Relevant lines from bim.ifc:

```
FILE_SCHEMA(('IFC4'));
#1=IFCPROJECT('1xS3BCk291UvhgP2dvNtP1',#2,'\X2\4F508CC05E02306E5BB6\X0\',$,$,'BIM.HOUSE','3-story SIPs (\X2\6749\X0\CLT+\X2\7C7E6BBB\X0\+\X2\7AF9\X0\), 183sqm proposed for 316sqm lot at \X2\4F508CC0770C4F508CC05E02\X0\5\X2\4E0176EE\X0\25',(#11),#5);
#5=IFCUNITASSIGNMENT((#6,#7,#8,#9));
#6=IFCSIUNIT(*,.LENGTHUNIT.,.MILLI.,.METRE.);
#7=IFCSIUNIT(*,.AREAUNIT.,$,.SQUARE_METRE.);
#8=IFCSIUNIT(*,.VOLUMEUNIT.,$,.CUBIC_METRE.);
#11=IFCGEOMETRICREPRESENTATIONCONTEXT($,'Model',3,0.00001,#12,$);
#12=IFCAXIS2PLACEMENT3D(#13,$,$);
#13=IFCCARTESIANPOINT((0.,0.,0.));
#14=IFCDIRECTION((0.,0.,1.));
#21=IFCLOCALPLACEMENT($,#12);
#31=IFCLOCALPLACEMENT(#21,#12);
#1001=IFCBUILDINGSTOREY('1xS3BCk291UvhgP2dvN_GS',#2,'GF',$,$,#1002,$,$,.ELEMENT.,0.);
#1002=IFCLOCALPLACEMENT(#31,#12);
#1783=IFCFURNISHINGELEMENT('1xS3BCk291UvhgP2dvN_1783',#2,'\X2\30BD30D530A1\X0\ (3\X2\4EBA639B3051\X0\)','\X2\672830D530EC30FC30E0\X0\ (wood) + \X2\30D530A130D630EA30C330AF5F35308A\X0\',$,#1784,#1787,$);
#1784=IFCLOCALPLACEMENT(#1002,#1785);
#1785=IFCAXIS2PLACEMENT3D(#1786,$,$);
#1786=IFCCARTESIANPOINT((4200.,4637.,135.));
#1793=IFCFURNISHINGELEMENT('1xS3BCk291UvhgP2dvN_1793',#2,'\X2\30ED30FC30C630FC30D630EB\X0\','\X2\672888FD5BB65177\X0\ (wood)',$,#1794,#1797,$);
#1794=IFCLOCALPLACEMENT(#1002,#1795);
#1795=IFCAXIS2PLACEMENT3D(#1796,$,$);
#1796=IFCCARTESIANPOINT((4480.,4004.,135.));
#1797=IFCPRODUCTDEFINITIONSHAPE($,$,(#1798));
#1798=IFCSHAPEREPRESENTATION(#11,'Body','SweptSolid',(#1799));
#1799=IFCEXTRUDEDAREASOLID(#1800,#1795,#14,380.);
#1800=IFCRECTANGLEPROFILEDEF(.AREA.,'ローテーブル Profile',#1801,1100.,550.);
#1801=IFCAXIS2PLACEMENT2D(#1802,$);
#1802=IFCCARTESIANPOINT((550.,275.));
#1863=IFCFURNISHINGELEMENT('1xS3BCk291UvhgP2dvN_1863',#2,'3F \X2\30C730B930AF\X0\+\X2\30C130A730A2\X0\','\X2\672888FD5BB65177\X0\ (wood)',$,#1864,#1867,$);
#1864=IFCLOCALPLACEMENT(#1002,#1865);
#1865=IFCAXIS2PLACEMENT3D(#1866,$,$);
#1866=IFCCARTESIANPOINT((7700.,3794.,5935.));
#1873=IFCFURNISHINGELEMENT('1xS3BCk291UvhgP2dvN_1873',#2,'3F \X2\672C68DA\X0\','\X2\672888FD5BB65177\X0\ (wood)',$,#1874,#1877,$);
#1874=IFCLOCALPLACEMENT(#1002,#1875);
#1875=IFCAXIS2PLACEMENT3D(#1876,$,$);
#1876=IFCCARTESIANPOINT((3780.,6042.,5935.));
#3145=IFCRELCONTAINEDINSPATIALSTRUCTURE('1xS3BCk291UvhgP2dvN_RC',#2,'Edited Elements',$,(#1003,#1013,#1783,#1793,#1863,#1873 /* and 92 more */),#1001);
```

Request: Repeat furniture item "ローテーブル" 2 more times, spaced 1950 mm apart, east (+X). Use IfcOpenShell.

```python
import numpy as np
import ifcopenshell
import ifcopenshell.api.geometry
import ifcopenshell.api.root
import ifcopenshell.util.element
import ifcopenshell.util.placement
import ifcopenshell.util.unit

model = ifcopenshell.open("bim.ifc")
unit_scale = ifcopenshell.util.unit.calculate_unit_scale(model)


def reuse_history(source, copy):
    """copy_class also copies each property set's owner history, people and application; keep the originals."""
    for rel in copy.IsDefinedBy:
        if rel.is_a("IfcRelDefinesByProperties") and (history := rel.RelatingPropertyDefinition.OwnerHistory):
            rel.RelatingPropertyDefinition.OwnerHistory = source.OwnerHistory
            ifcopenshell.util.element.remove_deep2(model, history)


source = model.by_guid("1xS3BCk291UvhgP2dvN_1793")
base = ifcopenshell.util.placement.get_local_placement(source.ObjectPlacement)
step = np.array([1.0, 0.0, 0.0]) * 1.95 / unit_scale

for i in range(1, 3):
    copy = ifcopenshell.api.root.copy_class(model, product=source)
    copy.Representation = ifcopenshell.util.element.copy_deep(
        model, source.Representation, exclude=["IfcGeometricRepresentationContext", "IfcRepresentationMap"]
    )
    reuse_history(source, copy)
    matrix = base.copy()
    matrix[:3, 3] += i * step
    print("added at", matrix[:3, 3].round(3) + 0.0)
    ifcopenshell.api.geometry.edit_object_placement(model, product=copy, matrix=matrix, is_si=False)

model.write("bim_v2.ifc")
```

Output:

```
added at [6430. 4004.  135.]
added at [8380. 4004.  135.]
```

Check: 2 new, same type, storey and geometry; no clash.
